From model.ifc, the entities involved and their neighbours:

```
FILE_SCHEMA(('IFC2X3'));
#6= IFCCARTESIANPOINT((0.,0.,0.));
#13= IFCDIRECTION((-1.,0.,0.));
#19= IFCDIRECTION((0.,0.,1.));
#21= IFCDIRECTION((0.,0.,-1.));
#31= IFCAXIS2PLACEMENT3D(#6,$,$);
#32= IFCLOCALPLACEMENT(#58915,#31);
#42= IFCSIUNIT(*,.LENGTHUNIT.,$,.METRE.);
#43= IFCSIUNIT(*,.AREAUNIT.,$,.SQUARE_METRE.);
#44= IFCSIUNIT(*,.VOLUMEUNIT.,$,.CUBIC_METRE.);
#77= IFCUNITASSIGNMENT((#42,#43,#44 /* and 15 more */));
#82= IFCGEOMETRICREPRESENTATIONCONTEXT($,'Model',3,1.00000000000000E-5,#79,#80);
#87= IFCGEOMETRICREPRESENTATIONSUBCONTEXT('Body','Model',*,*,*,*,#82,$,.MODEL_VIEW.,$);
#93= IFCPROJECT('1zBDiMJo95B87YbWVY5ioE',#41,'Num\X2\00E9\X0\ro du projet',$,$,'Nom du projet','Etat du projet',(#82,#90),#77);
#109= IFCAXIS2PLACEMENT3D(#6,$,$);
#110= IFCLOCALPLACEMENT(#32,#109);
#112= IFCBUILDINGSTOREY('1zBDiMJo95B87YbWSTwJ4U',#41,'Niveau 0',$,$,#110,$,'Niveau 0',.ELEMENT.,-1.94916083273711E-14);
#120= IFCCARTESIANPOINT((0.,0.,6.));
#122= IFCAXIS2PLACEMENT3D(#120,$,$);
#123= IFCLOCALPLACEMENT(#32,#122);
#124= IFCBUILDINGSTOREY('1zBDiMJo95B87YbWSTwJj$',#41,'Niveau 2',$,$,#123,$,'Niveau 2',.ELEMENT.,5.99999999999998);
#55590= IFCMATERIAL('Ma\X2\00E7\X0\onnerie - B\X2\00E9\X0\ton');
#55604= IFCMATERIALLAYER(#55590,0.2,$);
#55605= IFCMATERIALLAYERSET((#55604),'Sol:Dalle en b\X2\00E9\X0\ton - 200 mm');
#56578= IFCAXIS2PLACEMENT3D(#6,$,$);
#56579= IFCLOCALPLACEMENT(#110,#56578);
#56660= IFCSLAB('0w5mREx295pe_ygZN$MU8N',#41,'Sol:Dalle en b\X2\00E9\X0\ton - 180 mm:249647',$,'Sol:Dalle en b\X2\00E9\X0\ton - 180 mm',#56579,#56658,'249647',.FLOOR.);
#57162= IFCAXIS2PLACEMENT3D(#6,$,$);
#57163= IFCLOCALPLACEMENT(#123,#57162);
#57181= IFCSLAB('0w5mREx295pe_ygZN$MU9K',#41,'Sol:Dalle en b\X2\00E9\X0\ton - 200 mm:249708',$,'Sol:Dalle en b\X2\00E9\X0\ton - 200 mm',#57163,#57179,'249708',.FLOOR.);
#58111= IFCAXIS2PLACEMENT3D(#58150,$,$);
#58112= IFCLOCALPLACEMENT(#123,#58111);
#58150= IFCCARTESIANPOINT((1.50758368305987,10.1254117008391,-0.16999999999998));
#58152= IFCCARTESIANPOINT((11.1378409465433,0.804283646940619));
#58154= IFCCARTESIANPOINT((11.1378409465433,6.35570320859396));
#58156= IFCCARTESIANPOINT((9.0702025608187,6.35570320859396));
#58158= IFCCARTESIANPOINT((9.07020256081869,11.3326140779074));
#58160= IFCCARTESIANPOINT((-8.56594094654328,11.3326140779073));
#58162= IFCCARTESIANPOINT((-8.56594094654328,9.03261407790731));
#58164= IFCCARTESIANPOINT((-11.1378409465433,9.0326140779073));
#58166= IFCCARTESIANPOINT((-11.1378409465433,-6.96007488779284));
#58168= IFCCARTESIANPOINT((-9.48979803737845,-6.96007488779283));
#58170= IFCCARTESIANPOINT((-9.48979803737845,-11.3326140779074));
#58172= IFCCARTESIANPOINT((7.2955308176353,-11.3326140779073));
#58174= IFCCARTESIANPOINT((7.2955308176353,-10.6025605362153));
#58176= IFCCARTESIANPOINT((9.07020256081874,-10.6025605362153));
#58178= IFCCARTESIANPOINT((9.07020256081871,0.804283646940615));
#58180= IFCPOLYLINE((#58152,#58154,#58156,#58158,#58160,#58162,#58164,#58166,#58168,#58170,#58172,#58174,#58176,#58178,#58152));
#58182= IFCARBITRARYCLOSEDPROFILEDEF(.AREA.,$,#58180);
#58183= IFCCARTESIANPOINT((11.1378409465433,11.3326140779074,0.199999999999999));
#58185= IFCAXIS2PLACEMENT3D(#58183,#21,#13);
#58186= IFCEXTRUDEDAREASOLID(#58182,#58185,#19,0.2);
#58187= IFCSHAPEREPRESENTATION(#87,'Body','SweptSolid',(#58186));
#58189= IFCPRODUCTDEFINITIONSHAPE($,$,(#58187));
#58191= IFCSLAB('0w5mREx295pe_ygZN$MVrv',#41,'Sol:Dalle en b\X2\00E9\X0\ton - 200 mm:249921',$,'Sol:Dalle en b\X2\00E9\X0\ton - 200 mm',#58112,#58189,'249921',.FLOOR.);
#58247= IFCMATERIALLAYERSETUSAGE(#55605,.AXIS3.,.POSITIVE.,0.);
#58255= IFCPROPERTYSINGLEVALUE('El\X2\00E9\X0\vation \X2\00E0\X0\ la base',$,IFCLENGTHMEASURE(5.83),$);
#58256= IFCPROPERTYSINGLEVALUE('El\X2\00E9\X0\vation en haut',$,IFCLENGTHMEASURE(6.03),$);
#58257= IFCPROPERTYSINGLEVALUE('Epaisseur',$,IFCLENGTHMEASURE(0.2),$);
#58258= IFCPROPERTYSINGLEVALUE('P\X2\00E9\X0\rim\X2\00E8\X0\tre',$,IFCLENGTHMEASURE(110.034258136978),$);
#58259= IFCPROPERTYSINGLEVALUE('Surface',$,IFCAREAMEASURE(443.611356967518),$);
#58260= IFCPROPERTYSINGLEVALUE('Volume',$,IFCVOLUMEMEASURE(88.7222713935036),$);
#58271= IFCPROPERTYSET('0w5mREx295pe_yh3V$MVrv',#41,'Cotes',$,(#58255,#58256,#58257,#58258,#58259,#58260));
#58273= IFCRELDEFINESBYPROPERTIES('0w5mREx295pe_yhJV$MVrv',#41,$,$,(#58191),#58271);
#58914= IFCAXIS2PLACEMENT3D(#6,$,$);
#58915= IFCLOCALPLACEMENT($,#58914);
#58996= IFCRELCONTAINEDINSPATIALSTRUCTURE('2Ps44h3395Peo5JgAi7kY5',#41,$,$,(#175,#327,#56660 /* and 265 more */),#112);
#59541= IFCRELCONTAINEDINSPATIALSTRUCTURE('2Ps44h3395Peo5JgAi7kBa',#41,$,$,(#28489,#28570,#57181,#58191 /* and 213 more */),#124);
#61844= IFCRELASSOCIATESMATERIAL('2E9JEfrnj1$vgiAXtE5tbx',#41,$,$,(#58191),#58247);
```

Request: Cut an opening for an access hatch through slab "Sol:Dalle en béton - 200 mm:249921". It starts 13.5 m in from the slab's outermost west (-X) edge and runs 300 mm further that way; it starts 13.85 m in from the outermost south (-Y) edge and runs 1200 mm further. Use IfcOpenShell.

```python
import numpy as np
import ifcopenshell
import ifcopenshell.api.feature
import ifcopenshell.api.geometry
import ifcopenshell.api.pset
import ifcopenshell.api.root
import ifcopenshell.geom
import ifcopenshell.util.element
import ifcopenshell.util.placement
import ifcopenshell.util.representation
import ifcopenshell.util.shape
import ifcopenshell.util.unit

model = ifcopenshell.open("model.ifc")
unit_scale = ifcopenshell.util.unit.calculate_unit_scale(model)
area_scale = ifcopenshell.util.unit.calculate_unit_scale(model, "AREAUNIT")
volume_scale = ifcopenshell.util.unit.calculate_unit_scale(model, "VOLUMEUNIT")
settings = ifcopenshell.geom.settings()


def volume(element):
    """Net volume in cubic metres, openings subtracted."""
    shape = ifcopenshell.geom.create_shape(settings, element)
    return ifcopenshell.util.shape.get_volume(shape.geometry)


slab = model.by_guid("0w5mREx295pe_ygZN$MVrv")
before = volume(slab)

# Extent in the slab's own axes, in metres. The edges named are its -X and -Y sides.
slab_shape = ifcopenshell.geom.create_shape(settings, slab)
vertices = ifcopenshell.util.shape.get_vertices(slab_shape.geometry)
x_min, y_min, bottom = vertices.min(axis=0)
top = vertices[:, 2].max()

opening = ifcopenshell.api.root.create_entity(model, ifc_class="IfcOpeningElement", name="Access hatch opening")
context = ifcopenshell.util.representation.get_context(model, "Model", "Body", "MODEL_VIEW")
width, depth = 0.3, 1.2
outline = [(0.0, 0.0), (width, 0.0), (width, depth), (0.0, depth), (0.0, 0.0)]
# Overshoot both faces by 50 mm so the cut is clean.
shape = ifcopenshell.api.geometry.add_slab_representation(
    model, context=context, depth=top - bottom + 0.1, polyline=outline
)
ifcopenshell.api.geometry.assign_representation(model, product=opening, representation=shape)

matrix = ifcopenshell.util.placement.get_local_placement(slab.ObjectPlacement)
matrix[:, 3] = matrix @ np.append(np.array([x_min + 13.5, y_min + 13.85, bottom - 0.05]) / unit_scale, 1.0)
ifcopenshell.api.geometry.edit_object_placement(model, product=opening, matrix=matrix, is_si=False)
ifcopenshell.api.feature.add_feature(model, feature=opening, element=slab)

after = volume(slab)

# Update the slab's stored quantities.
pset = model.by_id(ifcopenshell.util.element.get_pset(slab, "Cotes", should_inherit=False)["id"])
ifcopenshell.api.pset.edit_pset(model, pset=pset, properties={
    "Surface": model.create_entity("IfcAreaMeasure", after / (top - bottom) / area_scale),
    "Volume": model.create_entity("IfcVolumeMeasure", after / volume_scale),
})

print(f"slab volume {before:.3f} -> {after:.3f} m3")

model.write("model_edited.ifc")
```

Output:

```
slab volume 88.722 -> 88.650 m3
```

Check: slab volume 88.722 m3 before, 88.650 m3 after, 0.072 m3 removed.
